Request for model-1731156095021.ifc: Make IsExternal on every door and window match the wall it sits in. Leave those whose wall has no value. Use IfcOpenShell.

First a look at what the model holds.

```python
import ifcopenshell
import ifcopenshell.util.element

model = ifcopenshell.open("model-1731156095021.ifc")
print(model.schema)
seen = {}
for e in model.by_type("IfcDoor") + model.by_type("IfcWindow"):
    if not e.FillsVoids:
        continue
    host = e.FillsVoids[0].RelatingOpeningElement.VoidsElements[0].RelatingBuildingElement
    own = ifcopenshell.util.element.get_pset(e, f"Pset_{e.is_a()[3:].removesuffix('StandardCase')}Common", "IsExternal")
    wall = ifcopenshell.util.element.get_pset(host, "Pset_WallCommon", "IsExternal")
    seen[e.is_a(), own, wall] = seen.get((e.is_a(), own, wall), 0) + 1
for (cls, own, wall), count in sorted(seen.items(), key=str):
    print(count, cls, "IsExternal:", own, "| host wall:", wall)
```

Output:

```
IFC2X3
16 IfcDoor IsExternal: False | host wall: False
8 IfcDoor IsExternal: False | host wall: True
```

```python
import ifcopenshell
import ifcopenshell.api.pset
import ifcopenshell.util.element

model = ifcopenshell.open("model-1731156095021.ifc")

count = 0
for ifc_class, pset_name in (("IfcDoor", "Pset_DoorCommon"), ("IfcWindow", "Pset_WindowCommon")):
    for e in model.by_type(ifc_class):
        if not e.FillsVoids:
            continue
        host = e.FillsVoids[0].RelatingOpeningElement.VoidsElements[0].RelatingBuildingElement
        external = ifcopenshell.util.element.get_pset(host, "Pset_WallCommon", "IsExternal")
        if external is None or ifcopenshell.util.element.get_pset(e, pset_name, "IsExternal") == external:
            continue
        pset = ifcopenshell.api.pset.add_pset(model, product=e, name=pset_name)
        ifcopenshell.api.pset.edit_pset(model, pset=pset, properties={"IsExternal": external})
        count += 1

print(count, "updated")

model.write("model-1731156095021_v2.ifc")
```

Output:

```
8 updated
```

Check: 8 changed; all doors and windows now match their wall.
